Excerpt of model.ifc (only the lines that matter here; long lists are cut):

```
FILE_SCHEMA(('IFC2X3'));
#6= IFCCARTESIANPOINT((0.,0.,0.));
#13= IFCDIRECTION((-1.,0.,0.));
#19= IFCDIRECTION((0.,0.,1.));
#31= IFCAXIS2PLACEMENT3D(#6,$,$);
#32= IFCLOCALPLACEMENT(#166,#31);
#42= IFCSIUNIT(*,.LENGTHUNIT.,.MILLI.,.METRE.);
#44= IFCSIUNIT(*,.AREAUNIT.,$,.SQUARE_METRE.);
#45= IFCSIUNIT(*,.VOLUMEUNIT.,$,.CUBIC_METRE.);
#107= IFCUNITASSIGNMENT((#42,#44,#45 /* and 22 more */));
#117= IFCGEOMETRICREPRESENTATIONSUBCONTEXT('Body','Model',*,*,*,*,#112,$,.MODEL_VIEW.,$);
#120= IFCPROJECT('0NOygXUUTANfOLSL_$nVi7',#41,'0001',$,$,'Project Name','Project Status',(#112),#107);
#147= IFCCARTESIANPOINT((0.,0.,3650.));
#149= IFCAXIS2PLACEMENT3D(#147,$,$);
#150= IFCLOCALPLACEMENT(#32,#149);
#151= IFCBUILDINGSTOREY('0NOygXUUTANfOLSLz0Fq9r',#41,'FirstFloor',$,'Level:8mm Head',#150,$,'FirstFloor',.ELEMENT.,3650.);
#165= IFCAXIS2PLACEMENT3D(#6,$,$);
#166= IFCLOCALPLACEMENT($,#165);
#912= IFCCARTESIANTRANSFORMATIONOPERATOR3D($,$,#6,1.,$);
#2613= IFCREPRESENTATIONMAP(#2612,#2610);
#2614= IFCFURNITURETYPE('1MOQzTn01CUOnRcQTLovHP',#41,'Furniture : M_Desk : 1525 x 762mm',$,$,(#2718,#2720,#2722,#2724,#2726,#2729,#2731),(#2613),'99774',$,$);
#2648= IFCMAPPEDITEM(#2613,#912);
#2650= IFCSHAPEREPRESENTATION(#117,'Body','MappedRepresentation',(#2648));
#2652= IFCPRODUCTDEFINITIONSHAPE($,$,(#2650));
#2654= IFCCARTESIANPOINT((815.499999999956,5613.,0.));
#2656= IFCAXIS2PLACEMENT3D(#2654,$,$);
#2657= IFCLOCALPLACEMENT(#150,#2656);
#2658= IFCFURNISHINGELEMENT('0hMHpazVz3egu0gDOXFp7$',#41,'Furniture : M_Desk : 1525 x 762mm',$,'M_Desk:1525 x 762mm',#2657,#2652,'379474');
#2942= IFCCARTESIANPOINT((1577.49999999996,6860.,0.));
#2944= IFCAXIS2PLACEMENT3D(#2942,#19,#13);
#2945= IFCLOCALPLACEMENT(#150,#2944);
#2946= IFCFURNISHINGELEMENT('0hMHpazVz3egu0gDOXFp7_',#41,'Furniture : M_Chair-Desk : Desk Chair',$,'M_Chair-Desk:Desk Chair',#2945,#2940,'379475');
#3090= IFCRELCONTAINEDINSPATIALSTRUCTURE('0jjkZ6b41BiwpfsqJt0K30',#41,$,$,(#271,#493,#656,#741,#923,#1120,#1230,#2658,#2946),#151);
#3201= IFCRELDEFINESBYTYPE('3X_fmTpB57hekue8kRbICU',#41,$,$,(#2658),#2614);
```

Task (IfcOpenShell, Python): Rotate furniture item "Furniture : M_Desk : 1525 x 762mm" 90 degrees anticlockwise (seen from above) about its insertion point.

```python
import ifcopenshell
import ifcopenshell.api.geometry
import ifcopenshell.util.placement

model = ifcopenshell.open("model.ifc")

item = model.by_guid("0hMHpazVz3egu0gDOXFp7$")
matrix = ifcopenshell.util.placement.get_local_placement(item.ObjectPlacement)
matrix = matrix @ ifcopenshell.util.placement.rotation(90, "Z")
ifcopenshell.api.geometry.edit_object_placement(model, product=item, matrix=matrix, is_si=False)

print(ifcopenshell.util.placement.get_local_placement(item.ObjectPlacement).round(3) + 0.0)

model.write("model_edited.ifc")
```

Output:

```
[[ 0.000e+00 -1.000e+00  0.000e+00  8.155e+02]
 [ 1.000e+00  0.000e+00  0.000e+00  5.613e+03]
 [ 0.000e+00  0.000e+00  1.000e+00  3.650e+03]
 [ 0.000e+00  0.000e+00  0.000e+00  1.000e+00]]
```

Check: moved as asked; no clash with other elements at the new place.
